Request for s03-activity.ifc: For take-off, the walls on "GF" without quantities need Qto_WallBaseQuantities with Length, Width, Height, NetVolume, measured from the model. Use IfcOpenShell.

First a look at what the model holds.

```python
import ifcopenshell
import ifcopenshell.util.element
import ifcopenshell.util.unit

model = ifcopenshell.open("s03-activity.ifc")
print(model.schema)
for unit_type in ("LENGTHUNIT", "AREAUNIT", "VOLUMEUNIT"):
    print(unit_type, ifcopenshell.util.unit.calculate_unit_scale(model, unit_type))
storey = next(s for s in model.by_type("IfcBuildingStorey") if s.Name == "GF")
walls = [e for e in ifcopenshell.util.element.get_decomposition(storey) if e.is_a("IfcWall")]
for e in sorted(walls, key=lambda e: e.id()):
    print(e.id(), e.is_a(), e.Name, list(ifcopenshell.util.element.get_psets(e, qtos_only=True)), sep=" | ")
```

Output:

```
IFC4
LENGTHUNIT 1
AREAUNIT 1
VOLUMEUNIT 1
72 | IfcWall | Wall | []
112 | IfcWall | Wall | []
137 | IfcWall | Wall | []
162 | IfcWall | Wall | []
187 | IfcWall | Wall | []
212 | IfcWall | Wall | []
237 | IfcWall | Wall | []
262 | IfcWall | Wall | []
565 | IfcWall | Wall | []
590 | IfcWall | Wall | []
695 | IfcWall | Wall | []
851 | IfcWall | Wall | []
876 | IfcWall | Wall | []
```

```python
import ifcopenshell
import ifcopenshell.api.pset
import ifcopenshell.geom
import ifcopenshell.util.element
import ifcopenshell.util.shape
import ifcopenshell.util.unit

model = ifcopenshell.open("s03-activity.ifc")
unit_scale = ifcopenshell.util.unit.calculate_unit_scale(model)
volume_scale = ifcopenshell.util.unit.calculate_unit_scale(model, "VOLUMEUNIT")
settings = ifcopenshell.geom.settings()

storey = next(s for s in model.by_type("IfcBuildingStorey") if s.Name == "GF")
walls = [e for e in ifcopenshell.util.element.get_decomposition(storey) if e.is_a("IfcWall")]

for e in sorted(walls, key=lambda e: e.id()):
    if ifcopenshell.util.element.get_psets(e, qtos_only=True, should_inherit=False):
        continue
    # Geometry comes back in metres, in the element's own axes.
    shape = ifcopenshell.geom.create_shape(settings, e)
    values = {
        "Length": ifcopenshell.util.shape.get_x(shape.geometry) / unit_scale,
        "Width": ifcopenshell.util.shape.get_y(shape.geometry) / unit_scale,
        "Height": ifcopenshell.util.shape.get_z(shape.geometry) / unit_scale,
        "NetVolume": ifcopenshell.util.shape.get_volume(shape.geometry) / volume_scale,
    }
    qto = ifcopenshell.api.pset.add_qto(model, product=e, name="Qto_WallBaseQuantities")
    ifcopenshell.api.pset.edit_qto(model, qto=qto, properties=values)
    print(e.id(), {k: round(v, 3) for k, v in values.items()})

model.write("s03-activity_v2.ifc")
```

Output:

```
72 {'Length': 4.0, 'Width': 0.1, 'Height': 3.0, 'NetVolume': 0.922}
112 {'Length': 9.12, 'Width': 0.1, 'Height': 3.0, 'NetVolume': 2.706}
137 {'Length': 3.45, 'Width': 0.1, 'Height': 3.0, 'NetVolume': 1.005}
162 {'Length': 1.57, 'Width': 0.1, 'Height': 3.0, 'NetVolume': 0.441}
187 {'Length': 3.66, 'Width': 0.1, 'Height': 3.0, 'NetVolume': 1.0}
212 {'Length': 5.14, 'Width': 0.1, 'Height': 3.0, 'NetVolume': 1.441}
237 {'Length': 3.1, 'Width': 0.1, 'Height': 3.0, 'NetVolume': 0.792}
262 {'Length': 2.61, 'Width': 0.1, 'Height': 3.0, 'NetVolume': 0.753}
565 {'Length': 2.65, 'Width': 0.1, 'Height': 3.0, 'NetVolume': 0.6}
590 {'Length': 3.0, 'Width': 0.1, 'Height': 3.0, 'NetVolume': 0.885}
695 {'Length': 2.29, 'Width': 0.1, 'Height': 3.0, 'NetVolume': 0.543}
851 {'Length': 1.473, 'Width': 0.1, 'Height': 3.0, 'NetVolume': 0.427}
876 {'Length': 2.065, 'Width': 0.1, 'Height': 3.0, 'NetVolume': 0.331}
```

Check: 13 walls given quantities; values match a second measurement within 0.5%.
